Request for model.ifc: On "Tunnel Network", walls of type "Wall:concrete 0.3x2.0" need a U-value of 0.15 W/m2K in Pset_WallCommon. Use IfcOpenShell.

First a look at what the model holds.

```python
import ifcopenshell
import ifcopenshell.util.element

model = ifcopenshell.open("model.ifc")
print(model.schema)
storey = next(s for s in model.by_type("IfcBuildingStorey") if s.Name == "Tunnel Network")
walls = [e for e in ifcopenshell.util.element.get_decomposition(storey) if e.is_a("IfcWall")]
seen = {}
for e in walls:
    element_type = ifcopenshell.util.element.get_type(e)
    key = (element_type.Name if element_type != e and element_type else None, ifcopenshell.util.element.get_pset(e, "Pset_WallCommon", "ThermalTransmittance"))
    seen[key] = seen.get(key, 0) + 1
for (name, value), count in sorted(seen.items(), key=str):
    print(count, "x", name, "|", value)
```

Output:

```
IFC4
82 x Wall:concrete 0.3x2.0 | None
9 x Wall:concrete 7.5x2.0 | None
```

```python
import ifcopenshell
import ifcopenshell.api.pset
import ifcopenshell.util.element

model = ifcopenshell.open("model.ifc")

storey = next(s for s in model.by_type("IfcBuildingStorey") if s.Name == "Tunnel Network")
walls = [e for e in ifcopenshell.util.element.get_decomposition(storey) if e.is_a("IfcWall")]

count = 0
for e in walls:
    element_type = ifcopenshell.util.element.get_type(e)
    if element_type in (None, e) or element_type.Name != "Wall:concrete 0.3x2.0":
        continue
    # add_pset returns the element's existing set when there is one.
    pset = ifcopenshell.api.pset.add_pset(model, product=e, name="Pset_WallCommon")
    ifcopenshell.api.pset.edit_pset(model, pset=pset, properties={"ThermalTransmittance": 0.15})
    count += 1

print(count, "walls updated")

model.write("model_edited.ifc")
```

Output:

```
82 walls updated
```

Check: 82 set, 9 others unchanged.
